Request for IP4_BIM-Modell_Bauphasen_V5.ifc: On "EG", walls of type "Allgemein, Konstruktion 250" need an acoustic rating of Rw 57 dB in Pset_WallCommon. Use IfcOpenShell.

First a look at what the model holds.

```python
import ifcopenshell
import ifcopenshell.util.element

model = ifcopenshell.open("IP4_BIM-Modell_Bauphasen_V5.ifc")
print(model.schema)
storey = next(s for s in model.by_type("IfcBuildingStorey") if s.Name == "EG")
walls = [e for e in ifcopenshell.util.element.get_decomposition(storey) if e.is_a("IfcWall")]
seen = {}
for e in walls:
    element_type = ifcopenshell.util.element.get_type(e)
    key = (element_type.Name if element_type != e and element_type else None, ifcopenshell.util.element.get_pset(e, "Pset_WallCommon", "AcousticRating"))
    seen[key] = seen.get(key, 0) + 1
for (name, value), count in sorted(seen.items(), key=str):
    print(count, "x", name, "|", value)
```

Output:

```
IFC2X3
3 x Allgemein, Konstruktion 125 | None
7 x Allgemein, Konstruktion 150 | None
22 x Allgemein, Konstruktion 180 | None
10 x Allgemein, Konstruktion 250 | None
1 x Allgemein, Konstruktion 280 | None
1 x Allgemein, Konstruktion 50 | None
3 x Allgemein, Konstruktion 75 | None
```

```python
import ifcopenshell
import ifcopenshell.api.pset
import ifcopenshell.util.element

model = ifcopenshell.open("IP4_BIM-Modell_Bauphasen_V5.ifc")

storey = next(s for s in model.by_type("IfcBuildingStorey") if s.Name == "EG")
walls = [e for e in ifcopenshell.util.element.get_decomposition(storey) if e.is_a("IfcWall")]

count = 0
for e in walls:
    element_type = ifcopenshell.util.element.get_type(e)
    if element_type in (None, e) or element_type.Name != "Allgemein, Konstruktion 250":
        continue
    # add_pset returns the element's existing set when there is one.
    pset = ifcopenshell.api.pset.add_pset(model, product=e, name="Pset_WallCommon")
    ifcopenshell.api.pset.edit_pset(model, pset=pset, properties={"AcousticRating": "Rw 57 dB"})
    count += 1

print(count, "walls updated")

model.write("IP4_BIM-Modell_Bauphasen_V5-out.ifc")
```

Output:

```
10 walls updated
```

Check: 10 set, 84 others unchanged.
